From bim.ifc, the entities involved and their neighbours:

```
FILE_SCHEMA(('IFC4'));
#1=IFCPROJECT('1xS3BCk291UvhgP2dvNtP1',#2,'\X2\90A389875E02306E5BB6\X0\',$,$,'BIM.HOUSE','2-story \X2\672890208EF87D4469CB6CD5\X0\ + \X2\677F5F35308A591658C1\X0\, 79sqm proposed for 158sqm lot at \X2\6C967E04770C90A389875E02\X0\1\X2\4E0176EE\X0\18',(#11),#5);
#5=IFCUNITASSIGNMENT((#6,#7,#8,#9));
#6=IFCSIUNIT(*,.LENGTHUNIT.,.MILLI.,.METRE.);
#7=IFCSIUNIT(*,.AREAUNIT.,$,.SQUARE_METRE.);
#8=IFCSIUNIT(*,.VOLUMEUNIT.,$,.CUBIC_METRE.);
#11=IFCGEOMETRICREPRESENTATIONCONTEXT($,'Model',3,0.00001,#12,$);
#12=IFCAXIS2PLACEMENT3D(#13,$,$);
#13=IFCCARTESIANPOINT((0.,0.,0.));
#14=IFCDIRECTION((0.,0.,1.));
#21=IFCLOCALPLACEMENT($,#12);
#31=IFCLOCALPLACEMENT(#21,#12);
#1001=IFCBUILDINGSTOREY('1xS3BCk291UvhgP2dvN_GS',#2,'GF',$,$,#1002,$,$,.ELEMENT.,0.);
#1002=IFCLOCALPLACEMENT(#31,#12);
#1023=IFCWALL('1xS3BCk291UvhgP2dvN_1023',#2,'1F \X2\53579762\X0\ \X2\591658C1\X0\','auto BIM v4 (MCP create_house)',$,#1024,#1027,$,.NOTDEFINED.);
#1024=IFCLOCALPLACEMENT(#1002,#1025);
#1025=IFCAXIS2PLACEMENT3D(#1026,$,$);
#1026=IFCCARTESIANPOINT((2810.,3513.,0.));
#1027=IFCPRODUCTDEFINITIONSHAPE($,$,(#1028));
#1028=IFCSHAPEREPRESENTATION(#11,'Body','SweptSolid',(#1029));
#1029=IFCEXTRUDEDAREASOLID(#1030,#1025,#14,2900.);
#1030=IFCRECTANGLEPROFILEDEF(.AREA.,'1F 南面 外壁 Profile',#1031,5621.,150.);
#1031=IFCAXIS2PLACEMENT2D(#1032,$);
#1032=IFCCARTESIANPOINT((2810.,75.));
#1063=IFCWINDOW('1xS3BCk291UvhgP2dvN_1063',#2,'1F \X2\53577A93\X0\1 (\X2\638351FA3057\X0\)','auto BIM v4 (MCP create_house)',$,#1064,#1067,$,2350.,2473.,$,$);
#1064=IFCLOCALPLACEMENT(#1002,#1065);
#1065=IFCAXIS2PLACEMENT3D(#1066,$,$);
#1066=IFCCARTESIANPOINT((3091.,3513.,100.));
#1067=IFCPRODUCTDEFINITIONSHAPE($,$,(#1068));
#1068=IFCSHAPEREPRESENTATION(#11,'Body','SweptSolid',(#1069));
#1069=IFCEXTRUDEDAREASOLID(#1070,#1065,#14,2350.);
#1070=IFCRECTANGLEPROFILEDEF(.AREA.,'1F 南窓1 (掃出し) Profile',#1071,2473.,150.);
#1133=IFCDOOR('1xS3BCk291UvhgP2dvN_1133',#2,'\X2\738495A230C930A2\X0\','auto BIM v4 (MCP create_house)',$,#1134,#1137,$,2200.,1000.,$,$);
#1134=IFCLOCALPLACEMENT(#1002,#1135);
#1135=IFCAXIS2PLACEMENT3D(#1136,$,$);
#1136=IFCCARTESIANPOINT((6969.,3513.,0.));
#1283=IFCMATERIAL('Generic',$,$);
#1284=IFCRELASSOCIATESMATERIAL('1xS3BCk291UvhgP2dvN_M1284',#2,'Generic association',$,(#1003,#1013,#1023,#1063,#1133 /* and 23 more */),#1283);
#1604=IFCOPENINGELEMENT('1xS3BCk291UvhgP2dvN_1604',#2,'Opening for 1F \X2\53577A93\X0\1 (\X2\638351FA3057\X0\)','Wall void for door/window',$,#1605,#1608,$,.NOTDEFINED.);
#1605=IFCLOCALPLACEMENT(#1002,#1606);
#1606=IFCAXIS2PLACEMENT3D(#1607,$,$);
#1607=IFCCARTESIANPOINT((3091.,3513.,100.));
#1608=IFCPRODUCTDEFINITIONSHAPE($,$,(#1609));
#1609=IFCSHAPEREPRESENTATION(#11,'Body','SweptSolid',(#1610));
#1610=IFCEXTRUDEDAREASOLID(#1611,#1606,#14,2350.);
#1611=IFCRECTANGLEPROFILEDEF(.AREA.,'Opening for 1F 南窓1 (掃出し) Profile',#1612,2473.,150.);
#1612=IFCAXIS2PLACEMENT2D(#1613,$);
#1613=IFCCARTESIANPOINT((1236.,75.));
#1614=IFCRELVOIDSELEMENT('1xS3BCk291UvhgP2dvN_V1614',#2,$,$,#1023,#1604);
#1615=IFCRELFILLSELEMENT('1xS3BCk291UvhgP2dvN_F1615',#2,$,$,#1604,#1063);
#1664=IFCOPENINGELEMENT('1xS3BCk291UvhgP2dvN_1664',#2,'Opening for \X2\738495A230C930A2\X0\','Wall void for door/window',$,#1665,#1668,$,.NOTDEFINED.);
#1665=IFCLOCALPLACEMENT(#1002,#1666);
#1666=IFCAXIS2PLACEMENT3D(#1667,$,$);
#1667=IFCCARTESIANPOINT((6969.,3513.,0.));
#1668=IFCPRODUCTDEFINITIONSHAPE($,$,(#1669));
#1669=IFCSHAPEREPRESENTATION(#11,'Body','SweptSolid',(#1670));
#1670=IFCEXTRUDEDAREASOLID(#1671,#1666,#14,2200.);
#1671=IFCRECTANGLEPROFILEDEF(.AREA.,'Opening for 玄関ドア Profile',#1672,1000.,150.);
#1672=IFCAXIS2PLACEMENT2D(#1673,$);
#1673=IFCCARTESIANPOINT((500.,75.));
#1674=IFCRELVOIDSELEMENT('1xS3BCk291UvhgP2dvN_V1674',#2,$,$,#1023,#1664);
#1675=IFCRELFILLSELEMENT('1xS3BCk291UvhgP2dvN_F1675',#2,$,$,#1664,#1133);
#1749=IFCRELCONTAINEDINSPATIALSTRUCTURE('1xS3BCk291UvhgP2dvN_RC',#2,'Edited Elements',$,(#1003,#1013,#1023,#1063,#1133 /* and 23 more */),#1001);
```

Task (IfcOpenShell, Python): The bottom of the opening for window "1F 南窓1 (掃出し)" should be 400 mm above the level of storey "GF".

```python
import numpy as np
import ifcopenshell
import ifcopenshell.api.geometry
import ifcopenshell.geom
import ifcopenshell.util.element
import ifcopenshell.util.placement
import ifcopenshell.util.shape
import ifcopenshell.util.unit

model = ifcopenshell.open("bim.ifc")
unit_scale = ifcopenshell.util.unit.calculate_unit_scale(model)

window = model.by_guid("1xS3BCk291UvhgP2dvN_1063")
opening = window.FillsVoids[0].RelatingOpeningElement
storey = ifcopenshell.util.element.get_container(window, ifc_class="IfcBuildingStorey")
level = ifcopenshell.util.placement.get_local_placement(storey.ObjectPlacement)[2, 3]

# The opening's origin need not be at the sill, so measure its lowest point.
shape = ifcopenshell.geom.create_shape(ifcopenshell.geom.settings(), opening)
bottom = ifcopenshell.util.shape.get_shape_bottom_elevation(shape, shape.geometry) / unit_scale
dz = level + 400.0 - bottom

shift = np.array([0.0, 0.0, dz])
# The window is not placed relative to its opening, so move both.
for product in (opening, window):
    matrix = ifcopenshell.util.placement.get_local_placement(product.ObjectPlacement)
    matrix[:3, 3] += shift
    ifcopenshell.api.geometry.edit_object_placement(model, product=product, matrix=matrix, is_si=False)

print(f"moved by {dz * unit_scale:+.3f} m")

model.write("bim_rev.ifc")
```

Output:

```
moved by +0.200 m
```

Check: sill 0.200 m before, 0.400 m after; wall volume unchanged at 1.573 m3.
